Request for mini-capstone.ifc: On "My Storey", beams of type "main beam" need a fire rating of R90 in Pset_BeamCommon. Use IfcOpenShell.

First a look at what the model holds.

```python
import ifcopenshell
import ifcopenshell.util.element

model = ifcopenshell.open("mini-capstone.ifc")
print(model.schema)
storey = next(s for s in model.by_type("IfcBuildingStorey") if s.Name == "My Storey")
beams = [e for e in ifcopenshell.util.element.get_decomposition(storey) if e.is_a("IfcBeam")]
seen = {}
for e in beams:
    element_type = ifcopenshell.util.element.get_type(e)
    key = (element_type.Name if element_type != e and element_type else None, ifcopenshell.util.element.get_pset(e, "Pset_BeamCommon", "FireRating"))
    seen[key] = seen.get(key, 0) + 1
for (name, value), count in sorted(seen.items(), key=str):
    print(count, "x", name, "|", value)
```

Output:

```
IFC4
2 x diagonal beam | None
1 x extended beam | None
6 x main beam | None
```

```python
import ifcopenshell
import ifcopenshell.api.pset
import ifcopenshell.util.element

model = ifcopenshell.open("mini-capstone.ifc")

storey = next(s for s in model.by_type("IfcBuildingStorey") if s.Name == "My Storey")
beams = [e for e in ifcopenshell.util.element.get_decomposition(storey) if e.is_a("IfcBeam")]

count = 0
for e in beams:
    element_type = ifcopenshell.util.element.get_type(e)
    if element_type in (None, e) or element_type.Name != "main beam":
        continue
    # add_pset returns the element's existing set when there is one.
    pset = ifcopenshell.api.pset.add_pset(model, product=e, name="Pset_BeamCommon")
    ifcopenshell.api.pset.edit_pset(model, pset=pset, properties={"FireRating": "R90"})
    count += 1

print(count, "beams updated")

model.write("mini-capstone_edited.ifc")
```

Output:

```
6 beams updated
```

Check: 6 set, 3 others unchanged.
